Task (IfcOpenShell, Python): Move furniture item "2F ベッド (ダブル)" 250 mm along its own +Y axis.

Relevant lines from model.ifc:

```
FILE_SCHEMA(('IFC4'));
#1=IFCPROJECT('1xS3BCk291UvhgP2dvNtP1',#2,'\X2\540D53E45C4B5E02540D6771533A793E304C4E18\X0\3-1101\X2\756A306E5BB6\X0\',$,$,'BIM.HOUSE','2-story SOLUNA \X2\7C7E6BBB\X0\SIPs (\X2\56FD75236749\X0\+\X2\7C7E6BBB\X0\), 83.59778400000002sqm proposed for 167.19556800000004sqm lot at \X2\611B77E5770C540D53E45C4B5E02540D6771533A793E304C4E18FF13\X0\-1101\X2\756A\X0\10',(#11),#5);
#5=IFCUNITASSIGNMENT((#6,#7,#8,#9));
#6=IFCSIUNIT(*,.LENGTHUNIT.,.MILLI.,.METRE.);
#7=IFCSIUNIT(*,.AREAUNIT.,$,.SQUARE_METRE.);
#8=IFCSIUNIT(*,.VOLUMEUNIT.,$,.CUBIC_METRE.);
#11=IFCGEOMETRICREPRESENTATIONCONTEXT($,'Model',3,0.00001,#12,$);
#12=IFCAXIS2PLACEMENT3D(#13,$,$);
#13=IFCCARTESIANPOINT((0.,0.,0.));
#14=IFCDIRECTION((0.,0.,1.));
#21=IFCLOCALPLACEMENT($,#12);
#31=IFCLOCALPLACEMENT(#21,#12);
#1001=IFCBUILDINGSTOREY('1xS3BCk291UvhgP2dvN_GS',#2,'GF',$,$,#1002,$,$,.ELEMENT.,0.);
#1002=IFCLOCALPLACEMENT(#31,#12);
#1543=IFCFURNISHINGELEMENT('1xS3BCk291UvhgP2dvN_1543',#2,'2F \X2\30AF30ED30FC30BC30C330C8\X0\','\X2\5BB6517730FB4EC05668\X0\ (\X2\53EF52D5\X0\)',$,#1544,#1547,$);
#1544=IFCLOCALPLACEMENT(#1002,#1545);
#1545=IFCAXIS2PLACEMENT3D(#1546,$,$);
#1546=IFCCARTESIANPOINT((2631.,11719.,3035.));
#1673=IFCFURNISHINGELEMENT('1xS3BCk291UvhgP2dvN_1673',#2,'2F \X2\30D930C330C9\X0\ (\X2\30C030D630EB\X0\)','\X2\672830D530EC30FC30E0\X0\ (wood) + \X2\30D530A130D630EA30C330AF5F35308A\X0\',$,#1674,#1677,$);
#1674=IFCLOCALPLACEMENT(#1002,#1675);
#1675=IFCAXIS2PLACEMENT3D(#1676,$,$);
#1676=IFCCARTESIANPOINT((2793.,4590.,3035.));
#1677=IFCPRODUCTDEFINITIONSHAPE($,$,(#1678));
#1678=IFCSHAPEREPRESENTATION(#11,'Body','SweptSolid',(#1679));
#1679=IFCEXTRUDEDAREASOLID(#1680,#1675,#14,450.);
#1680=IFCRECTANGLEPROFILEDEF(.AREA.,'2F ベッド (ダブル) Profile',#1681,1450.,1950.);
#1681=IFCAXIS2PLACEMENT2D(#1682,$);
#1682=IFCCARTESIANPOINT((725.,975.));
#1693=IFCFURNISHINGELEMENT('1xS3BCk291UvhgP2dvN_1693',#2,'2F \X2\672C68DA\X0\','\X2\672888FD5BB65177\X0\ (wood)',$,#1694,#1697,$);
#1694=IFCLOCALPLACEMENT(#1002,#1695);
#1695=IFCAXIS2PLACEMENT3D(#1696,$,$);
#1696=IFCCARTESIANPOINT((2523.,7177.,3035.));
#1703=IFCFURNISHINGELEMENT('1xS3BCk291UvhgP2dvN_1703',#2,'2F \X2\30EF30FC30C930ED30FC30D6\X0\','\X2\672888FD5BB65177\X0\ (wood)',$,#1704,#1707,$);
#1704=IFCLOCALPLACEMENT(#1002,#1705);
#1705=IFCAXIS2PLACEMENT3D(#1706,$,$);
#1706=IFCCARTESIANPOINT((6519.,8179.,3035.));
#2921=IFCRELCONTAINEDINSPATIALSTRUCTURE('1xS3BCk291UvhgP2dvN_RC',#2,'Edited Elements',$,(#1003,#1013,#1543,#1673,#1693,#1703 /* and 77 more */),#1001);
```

```python
import ifcopenshell
import ifcopenshell.api.geometry
import ifcopenshell.util.placement

model = ifcopenshell.open("model.ifc")

item = model.by_guid("1xS3BCk291UvhgP2dvN_1673")
matrix = ifcopenshell.util.placement.get_local_placement(item.ObjectPlacement)
matrix[:3, 3] += matrix[:3, 1] * 250.0
ifcopenshell.api.geometry.edit_object_placement(model, product=item, matrix=matrix, is_si=False)

print(ifcopenshell.util.placement.get_local_placement(item.ObjectPlacement).round(3) + 0.0)

model.write("model_edited.ifc")
```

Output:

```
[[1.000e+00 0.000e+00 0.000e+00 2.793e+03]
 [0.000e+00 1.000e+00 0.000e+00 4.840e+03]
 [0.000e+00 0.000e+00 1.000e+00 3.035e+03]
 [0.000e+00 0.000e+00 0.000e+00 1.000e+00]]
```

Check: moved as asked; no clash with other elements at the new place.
